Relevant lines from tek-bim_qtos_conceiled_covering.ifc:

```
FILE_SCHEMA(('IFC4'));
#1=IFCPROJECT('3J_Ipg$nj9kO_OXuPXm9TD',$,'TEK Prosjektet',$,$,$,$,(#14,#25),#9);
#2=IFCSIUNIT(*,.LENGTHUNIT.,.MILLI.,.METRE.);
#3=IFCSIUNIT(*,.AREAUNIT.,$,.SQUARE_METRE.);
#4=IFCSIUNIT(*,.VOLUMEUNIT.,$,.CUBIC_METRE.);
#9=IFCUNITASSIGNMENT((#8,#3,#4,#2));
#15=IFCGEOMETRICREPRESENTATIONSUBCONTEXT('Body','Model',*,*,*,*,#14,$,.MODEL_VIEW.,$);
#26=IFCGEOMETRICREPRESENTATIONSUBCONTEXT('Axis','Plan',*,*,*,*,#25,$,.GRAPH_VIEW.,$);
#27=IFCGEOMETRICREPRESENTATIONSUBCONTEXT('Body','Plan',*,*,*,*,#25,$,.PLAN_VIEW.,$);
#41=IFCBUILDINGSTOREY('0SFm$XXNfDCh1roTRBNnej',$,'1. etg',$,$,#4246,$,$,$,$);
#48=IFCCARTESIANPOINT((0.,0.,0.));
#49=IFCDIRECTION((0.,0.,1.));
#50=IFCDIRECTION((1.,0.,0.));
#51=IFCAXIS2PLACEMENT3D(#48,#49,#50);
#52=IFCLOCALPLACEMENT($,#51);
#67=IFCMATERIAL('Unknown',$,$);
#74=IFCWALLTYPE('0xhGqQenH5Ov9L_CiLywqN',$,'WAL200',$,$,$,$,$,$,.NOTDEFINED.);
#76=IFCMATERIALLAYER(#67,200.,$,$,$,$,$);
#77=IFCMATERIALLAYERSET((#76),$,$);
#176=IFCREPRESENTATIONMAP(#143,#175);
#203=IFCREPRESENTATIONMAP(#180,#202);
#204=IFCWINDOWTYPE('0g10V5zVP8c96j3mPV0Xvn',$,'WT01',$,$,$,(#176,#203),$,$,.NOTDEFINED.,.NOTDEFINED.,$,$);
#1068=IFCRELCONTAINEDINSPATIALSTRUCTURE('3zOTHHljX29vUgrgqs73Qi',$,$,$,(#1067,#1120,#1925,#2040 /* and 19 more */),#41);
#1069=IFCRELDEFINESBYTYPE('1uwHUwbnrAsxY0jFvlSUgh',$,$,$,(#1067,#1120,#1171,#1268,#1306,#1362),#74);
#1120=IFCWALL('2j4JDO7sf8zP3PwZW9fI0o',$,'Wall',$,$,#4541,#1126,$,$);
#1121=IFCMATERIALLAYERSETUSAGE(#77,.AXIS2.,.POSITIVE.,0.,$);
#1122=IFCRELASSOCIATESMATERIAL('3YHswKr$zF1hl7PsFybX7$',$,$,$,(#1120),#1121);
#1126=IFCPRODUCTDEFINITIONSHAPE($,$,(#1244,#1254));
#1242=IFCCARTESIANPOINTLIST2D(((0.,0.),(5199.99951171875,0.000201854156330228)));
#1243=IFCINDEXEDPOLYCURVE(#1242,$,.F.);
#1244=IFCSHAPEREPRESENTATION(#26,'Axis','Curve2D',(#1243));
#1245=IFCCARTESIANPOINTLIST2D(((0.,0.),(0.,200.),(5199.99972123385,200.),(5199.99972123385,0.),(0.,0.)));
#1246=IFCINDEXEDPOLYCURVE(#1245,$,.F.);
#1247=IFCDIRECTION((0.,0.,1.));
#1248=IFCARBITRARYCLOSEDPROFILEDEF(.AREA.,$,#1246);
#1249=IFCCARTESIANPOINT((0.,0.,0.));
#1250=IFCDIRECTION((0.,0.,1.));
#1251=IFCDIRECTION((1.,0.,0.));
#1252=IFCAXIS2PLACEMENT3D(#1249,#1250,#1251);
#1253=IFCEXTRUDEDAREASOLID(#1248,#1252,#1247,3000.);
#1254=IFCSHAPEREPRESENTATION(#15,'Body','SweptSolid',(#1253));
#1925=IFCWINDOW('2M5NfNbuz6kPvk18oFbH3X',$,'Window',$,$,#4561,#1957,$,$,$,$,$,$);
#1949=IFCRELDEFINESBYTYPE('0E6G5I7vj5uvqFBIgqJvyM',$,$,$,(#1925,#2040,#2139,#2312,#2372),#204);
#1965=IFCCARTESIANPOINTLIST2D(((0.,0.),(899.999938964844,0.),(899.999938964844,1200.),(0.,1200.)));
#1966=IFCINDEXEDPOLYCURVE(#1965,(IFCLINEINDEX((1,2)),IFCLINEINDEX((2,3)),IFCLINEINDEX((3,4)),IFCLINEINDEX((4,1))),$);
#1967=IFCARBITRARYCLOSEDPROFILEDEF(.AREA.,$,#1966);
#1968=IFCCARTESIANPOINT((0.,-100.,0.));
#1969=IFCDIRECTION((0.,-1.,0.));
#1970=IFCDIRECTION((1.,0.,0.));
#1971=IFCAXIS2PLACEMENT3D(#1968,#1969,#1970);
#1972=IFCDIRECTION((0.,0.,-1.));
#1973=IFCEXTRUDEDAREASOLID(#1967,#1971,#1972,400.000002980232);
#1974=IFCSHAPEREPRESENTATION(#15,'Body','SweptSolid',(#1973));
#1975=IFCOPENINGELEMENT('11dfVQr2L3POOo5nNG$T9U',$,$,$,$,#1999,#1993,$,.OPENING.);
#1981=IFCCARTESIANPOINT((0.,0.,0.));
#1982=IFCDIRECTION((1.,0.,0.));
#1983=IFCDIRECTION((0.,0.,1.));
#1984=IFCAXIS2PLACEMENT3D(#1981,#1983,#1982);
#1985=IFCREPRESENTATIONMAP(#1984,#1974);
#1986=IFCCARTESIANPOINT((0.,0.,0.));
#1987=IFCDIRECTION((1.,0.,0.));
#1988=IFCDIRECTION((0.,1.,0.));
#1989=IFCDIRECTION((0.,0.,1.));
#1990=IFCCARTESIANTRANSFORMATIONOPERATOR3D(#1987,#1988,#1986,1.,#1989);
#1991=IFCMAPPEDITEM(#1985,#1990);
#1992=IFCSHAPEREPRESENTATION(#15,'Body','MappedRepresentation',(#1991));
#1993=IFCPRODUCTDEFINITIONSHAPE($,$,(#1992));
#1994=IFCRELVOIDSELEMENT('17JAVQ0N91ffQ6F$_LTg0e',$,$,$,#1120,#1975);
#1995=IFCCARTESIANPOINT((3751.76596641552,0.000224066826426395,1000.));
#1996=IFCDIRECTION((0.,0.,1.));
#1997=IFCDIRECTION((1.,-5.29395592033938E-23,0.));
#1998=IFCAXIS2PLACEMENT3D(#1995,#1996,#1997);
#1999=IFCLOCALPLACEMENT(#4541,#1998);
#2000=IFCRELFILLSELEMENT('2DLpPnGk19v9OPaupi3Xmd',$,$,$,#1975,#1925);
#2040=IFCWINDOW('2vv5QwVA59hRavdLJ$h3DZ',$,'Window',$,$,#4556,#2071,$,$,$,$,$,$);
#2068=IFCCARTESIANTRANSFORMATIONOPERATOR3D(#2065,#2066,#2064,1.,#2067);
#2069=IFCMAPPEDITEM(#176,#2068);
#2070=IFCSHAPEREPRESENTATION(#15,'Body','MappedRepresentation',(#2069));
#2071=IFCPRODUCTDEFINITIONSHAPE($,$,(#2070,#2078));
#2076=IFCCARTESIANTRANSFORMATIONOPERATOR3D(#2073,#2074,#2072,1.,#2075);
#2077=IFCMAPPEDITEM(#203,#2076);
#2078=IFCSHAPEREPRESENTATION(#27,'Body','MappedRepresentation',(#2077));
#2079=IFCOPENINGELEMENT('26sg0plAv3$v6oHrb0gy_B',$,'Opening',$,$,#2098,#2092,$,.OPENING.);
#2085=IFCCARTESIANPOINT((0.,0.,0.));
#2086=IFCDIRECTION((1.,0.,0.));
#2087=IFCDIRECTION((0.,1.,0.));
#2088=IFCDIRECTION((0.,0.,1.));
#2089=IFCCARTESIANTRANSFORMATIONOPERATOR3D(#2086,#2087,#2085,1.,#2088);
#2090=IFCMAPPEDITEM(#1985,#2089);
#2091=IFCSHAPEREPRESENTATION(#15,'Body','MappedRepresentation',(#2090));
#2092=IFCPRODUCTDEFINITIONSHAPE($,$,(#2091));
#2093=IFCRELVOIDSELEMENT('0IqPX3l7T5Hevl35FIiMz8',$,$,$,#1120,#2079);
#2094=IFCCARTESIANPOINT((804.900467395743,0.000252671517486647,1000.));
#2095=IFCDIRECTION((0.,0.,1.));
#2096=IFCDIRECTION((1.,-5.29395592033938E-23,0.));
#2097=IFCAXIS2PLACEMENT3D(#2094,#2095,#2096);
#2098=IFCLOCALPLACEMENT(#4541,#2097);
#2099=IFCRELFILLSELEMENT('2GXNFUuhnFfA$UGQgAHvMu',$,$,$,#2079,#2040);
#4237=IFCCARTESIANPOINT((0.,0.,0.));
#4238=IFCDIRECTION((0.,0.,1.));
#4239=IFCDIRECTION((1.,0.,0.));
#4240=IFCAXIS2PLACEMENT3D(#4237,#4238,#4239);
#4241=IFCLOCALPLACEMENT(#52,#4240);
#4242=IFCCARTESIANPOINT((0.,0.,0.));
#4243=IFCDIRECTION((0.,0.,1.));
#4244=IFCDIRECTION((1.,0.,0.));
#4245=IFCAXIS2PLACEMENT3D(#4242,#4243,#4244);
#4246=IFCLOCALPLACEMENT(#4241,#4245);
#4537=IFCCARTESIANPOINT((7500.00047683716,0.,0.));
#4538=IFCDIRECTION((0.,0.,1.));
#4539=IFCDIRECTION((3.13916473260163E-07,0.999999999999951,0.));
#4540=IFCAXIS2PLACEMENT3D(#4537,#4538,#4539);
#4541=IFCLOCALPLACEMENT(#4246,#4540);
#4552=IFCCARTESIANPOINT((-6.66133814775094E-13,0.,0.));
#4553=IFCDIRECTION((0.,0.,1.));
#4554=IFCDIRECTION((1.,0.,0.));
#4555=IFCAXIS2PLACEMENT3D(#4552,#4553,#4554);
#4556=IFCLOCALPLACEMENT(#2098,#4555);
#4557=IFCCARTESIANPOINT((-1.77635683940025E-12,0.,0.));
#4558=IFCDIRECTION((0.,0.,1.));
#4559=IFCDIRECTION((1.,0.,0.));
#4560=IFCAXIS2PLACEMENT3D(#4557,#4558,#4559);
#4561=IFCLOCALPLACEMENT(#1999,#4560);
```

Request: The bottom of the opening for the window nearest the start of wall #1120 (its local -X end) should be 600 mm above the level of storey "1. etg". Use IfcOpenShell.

```python
import numpy as np
import ifcopenshell
import ifcopenshell.api.geometry
import ifcopenshell.geom
import ifcopenshell.util.element
import ifcopenshell.util.placement
import ifcopenshell.util.shape
import ifcopenshell.util.unit

model = ifcopenshell.open("tek-bim_qtos_conceiled_covering.ifc")
unit_scale = ifcopenshell.util.unit.calculate_unit_scale(model)

window = model.by_id(2040)
opening = window.FillsVoids[0].RelatingOpeningElement
storey = ifcopenshell.util.element.get_container(window, ifc_class="IfcBuildingStorey")
level = ifcopenshell.util.placement.get_local_placement(storey.ObjectPlacement)[2, 3]

# The opening's origin need not be at the sill, so measure its lowest point.
shape = ifcopenshell.geom.create_shape(ifcopenshell.geom.settings(), opening)
bottom = ifcopenshell.util.shape.get_shape_bottom_elevation(shape, shape.geometry) / unit_scale
dz = level + 0.6 / unit_scale - bottom

shift = np.array([0.0, 0.0, dz])
# The window is placed relative to its opening, so it follows when the opening moves.
matrix = ifcopenshell.util.placement.get_local_placement(opening.ObjectPlacement)
matrix[:3, 3] += shift
ifcopenshell.api.geometry.edit_object_placement(
    model, product=opening, matrix=matrix, is_si=False, should_transform_children=True
)

print(f"moved by {dz * unit_scale:+.3f} m")

model.write("tek-bim_qtos_conceiled_covering_v2.ifc")
```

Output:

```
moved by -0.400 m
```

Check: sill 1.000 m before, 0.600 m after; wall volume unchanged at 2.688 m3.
